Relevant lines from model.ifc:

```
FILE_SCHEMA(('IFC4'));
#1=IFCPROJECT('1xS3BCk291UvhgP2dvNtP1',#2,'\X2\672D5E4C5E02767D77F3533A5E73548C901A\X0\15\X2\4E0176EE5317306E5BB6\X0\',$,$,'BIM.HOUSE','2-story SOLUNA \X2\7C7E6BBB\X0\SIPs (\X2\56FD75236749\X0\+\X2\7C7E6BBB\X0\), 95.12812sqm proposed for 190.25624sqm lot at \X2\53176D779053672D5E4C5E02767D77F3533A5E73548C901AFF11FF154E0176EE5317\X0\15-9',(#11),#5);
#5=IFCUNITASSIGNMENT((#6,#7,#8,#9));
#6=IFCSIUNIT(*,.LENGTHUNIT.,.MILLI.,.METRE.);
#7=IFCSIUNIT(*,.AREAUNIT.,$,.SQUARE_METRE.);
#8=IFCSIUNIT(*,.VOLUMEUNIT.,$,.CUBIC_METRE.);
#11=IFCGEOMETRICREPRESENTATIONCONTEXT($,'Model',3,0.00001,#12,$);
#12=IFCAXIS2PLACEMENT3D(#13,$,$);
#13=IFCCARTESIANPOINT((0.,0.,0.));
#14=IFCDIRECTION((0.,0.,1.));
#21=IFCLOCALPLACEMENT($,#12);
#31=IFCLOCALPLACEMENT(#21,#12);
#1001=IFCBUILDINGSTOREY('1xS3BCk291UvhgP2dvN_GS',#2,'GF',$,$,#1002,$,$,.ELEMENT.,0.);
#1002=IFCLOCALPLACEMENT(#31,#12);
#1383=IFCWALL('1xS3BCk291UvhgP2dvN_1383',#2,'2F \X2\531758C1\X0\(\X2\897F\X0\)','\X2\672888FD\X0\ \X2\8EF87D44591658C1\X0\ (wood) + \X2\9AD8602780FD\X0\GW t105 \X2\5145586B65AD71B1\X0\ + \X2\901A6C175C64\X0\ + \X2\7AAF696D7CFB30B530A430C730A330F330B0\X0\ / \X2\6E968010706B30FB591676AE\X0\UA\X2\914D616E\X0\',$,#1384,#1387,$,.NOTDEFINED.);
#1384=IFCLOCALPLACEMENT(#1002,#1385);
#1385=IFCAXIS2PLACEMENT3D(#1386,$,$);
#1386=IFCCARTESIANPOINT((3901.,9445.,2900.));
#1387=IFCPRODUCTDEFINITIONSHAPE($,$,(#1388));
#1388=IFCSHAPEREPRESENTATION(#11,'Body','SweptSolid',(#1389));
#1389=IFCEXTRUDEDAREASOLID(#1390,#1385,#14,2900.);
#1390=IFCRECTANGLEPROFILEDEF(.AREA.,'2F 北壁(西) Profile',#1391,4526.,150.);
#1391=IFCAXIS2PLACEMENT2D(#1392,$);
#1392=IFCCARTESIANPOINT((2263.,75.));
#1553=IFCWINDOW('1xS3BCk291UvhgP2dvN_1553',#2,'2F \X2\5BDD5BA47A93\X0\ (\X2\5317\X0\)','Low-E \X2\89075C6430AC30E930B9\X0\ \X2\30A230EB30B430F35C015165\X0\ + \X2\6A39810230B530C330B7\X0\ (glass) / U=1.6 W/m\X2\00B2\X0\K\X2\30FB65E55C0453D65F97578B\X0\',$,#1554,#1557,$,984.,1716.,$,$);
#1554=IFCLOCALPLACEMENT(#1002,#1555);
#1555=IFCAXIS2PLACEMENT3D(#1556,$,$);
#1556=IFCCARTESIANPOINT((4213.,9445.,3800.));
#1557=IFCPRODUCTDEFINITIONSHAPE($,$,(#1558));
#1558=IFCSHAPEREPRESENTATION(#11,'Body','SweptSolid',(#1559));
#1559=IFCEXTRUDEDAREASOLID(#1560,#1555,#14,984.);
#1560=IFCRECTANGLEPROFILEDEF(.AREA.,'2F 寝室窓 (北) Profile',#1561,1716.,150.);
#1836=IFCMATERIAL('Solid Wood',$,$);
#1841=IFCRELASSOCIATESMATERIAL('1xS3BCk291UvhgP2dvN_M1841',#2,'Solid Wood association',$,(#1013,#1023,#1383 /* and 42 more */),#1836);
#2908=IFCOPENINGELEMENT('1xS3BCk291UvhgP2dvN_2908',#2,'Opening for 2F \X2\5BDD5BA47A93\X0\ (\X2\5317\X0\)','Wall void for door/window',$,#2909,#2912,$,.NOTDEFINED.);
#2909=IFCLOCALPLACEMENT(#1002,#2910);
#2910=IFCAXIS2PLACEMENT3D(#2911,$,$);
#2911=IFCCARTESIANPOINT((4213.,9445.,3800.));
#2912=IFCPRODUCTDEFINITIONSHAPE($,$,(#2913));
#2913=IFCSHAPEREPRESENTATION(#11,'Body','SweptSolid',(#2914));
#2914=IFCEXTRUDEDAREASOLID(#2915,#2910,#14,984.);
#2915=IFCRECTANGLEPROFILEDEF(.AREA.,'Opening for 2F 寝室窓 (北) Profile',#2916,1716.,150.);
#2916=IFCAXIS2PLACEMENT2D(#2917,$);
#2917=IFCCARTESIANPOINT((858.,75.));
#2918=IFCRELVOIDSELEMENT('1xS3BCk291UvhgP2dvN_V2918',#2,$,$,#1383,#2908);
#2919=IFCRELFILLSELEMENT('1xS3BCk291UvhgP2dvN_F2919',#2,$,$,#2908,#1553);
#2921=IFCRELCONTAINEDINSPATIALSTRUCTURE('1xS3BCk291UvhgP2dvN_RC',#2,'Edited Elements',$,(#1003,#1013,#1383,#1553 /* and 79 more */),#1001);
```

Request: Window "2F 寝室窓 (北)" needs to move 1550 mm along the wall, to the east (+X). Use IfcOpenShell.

```python
import ifcopenshell
import ifcopenshell.api.geometry
import ifcopenshell.util.placement
import ifcopenshell.util.unit

model = ifcopenshell.open("model.ifc")
unit_scale = ifcopenshell.util.unit.calculate_unit_scale(model)

window = model.by_guid("1xS3BCk291UvhgP2dvN_1553")
opening = window.FillsVoids[0].RelatingOpeningElement
wall = opening.VoidsElements[0].RelatingBuildingElement

wall_matrix = ifcopenshell.util.placement.get_local_placement(wall.ObjectPlacement)
shift = wall_matrix[:3, 0] * 1.55 / unit_scale
before = ifcopenshell.util.placement.get_local_placement(window.ObjectPlacement)[:3, 3].copy()

# The window is not placed relative to its opening, so move both.
for product in (opening, window):
    matrix = ifcopenshell.util.placement.get_local_placement(product.ObjectPlacement)
    matrix[:3, 3] += shift
    ifcopenshell.api.geometry.edit_object_placement(model, product=product, matrix=matrix, is_si=False)

after = ifcopenshell.util.placement.get_local_placement(window.ObjectPlacement)[:3, 3]
print("window moved by", (after - before).round(3) + 0.0)

model.write("model_v2.ifc")
```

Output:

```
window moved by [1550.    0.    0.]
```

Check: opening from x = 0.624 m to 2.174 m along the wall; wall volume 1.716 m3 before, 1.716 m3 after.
